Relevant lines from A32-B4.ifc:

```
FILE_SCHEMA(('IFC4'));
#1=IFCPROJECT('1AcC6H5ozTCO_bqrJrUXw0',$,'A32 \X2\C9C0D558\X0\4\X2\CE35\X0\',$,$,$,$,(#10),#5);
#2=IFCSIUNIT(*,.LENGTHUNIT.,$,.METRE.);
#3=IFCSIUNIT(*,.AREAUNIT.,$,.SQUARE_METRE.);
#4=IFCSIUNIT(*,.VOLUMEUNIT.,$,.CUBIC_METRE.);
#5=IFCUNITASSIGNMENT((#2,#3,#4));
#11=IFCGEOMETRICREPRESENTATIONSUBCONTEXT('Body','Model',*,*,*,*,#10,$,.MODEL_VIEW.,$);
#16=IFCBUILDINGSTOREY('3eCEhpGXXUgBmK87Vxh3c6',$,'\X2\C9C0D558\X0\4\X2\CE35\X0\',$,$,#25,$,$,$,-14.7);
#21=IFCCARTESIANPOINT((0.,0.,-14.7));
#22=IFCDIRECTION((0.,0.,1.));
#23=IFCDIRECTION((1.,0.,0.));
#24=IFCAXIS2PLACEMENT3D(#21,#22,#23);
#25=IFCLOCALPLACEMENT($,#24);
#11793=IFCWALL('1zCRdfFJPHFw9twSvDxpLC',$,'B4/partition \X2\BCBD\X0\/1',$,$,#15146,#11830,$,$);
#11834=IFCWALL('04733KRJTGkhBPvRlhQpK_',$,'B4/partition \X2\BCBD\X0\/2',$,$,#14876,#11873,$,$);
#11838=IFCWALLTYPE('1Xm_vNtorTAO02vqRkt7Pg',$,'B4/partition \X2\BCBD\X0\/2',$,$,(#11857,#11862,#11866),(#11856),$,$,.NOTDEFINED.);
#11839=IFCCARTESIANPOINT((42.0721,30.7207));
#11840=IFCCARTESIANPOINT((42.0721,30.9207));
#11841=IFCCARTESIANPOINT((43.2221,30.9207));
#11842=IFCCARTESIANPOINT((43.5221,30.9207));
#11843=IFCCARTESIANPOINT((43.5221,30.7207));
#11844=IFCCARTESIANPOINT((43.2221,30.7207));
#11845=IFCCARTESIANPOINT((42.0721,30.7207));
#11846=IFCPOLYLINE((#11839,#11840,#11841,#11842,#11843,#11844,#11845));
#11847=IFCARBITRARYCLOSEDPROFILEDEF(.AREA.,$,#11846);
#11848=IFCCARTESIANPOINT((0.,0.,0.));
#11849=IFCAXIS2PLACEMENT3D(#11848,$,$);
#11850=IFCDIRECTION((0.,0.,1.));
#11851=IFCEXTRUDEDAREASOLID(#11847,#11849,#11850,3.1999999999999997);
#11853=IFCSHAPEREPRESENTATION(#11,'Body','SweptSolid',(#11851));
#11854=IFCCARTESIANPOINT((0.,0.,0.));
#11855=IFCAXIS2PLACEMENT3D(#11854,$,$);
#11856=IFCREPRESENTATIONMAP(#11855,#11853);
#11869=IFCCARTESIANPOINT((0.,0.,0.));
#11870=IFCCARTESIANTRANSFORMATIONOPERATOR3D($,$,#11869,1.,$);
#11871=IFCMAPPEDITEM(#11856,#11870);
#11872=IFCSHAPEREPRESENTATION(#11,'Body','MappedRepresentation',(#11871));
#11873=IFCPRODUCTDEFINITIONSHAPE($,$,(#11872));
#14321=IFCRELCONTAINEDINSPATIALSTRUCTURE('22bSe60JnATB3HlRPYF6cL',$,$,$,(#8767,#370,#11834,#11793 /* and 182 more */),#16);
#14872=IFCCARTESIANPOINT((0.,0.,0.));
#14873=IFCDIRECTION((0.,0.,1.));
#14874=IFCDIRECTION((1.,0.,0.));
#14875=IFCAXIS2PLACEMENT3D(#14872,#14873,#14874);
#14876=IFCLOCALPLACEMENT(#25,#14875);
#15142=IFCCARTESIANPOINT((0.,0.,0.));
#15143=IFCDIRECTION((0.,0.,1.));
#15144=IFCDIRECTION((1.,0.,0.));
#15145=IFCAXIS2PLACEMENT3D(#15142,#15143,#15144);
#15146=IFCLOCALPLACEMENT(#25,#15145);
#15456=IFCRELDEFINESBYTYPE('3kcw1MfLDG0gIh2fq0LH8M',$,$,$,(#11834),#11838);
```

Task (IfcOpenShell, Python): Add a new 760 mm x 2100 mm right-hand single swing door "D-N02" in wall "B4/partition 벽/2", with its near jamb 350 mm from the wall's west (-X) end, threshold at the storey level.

```python
import numpy as np
import ifcopenshell
import ifcopenshell.api.feature
import ifcopenshell.api.geometry
import ifcopenshell.api.root
import ifcopenshell.api.spatial
import ifcopenshell.geom
import ifcopenshell.util.element
import ifcopenshell.util.placement
import ifcopenshell.util.representation
import ifcopenshell.util.shape
import ifcopenshell.util.unit

model = ifcopenshell.open("A32-B4.ifc")
unit_scale = ifcopenshell.util.unit.calculate_unit_scale(model)
settings = ifcopenshell.geom.settings()


def volume(element):
    """Net volume in cubic metres, openings subtracted."""
    shape = ifcopenshell.geom.create_shape(settings, element)
    return ifcopenshell.util.shape.get_volume(shape.geometry)


wall = model.by_id(11834)
storey = ifcopenshell.util.element.get_container(wall, ifc_class="IfcBuildingStorey")
context = ifcopenshell.util.representation.get_context(model, "Model", "Body", "MODEL_VIEW")
before = volume(wall)

width, height, from_end, sill = 0.76, 2.1, 0.35, 0.0  # metres

# The wall runs along its own X axis, and the end named is its -X end.
wall_shape = ifcopenshell.geom.create_shape(settings, wall)
x, y, z = ifcopenshell.util.shape.get_vertices(wall_shape.geometry).T
start = x.min() + from_end
face, thickness = float(y.min()), float(y.max() - y.min())
wall_matrix = ifcopenshell.util.placement.get_local_placement(wall.ObjectPlacement)
level = ifcopenshell.util.placement.get_local_placement(storey.ObjectPlacement)[2, 3]


def in_wall(x, y):
    """Placement at x, y metres in the wall's axes, at sill height."""
    matrix = wall_matrix.copy()
    matrix[:, 3] = wall_matrix @ np.array([x / unit_scale, y / unit_scale, 0.0, 1.0])
    matrix[2, 3] = level + sill / unit_scale
    return matrix


# Opening: a box that overshoots both wall faces by 50 mm.
opening = ifcopenshell.api.root.create_entity(model, ifc_class="IfcOpeningElement", predefined_type="OPENING")
box = ifcopenshell.api.geometry.add_wall_representation(
    model, context=context, length=width, height=height, thickness=thickness + 0.1
)
ifcopenshell.api.geometry.assign_representation(model, product=opening, representation=box)
ifcopenshell.api.geometry.edit_object_placement(model, product=opening, matrix=in_wall(start, face - 0.05), is_si=False)
ifcopenshell.api.feature.add_feature(model, feature=opening, element=wall)

door = ifcopenshell.api.root.create_entity(model, ifc_class="IfcDoor", name="D-N02", predefined_type="DOOR")
door.OverallWidth, door.OverallHeight = width / unit_scale, height / unit_scale
door.OperationType = "SINGLE_SWING_RIGHT"
body = ifcopenshell.api.geometry.add_door_representation(
    model,
    context=context,
    overall_width=door.OverallWidth,
    overall_height=door.OverallHeight,
    operation_type="SINGLE_SWING_RIGHT",
    lining_properties={"LiningDepth": thickness / unit_scale, "ThresholdDepth": thickness / unit_scale},
)
ifcopenshell.api.geometry.assign_representation(model, product=door, representation=body)
ifcopenshell.api.spatial.assign_container(model, products=[door], relating_structure=storey)
ifcopenshell.api.feature.add_filling(model, opening=opening, element=door)

# The lining spans the wall, so the door starts at the wall face.
ifcopenshell.api.geometry.edit_object_placement(model, product=door, matrix=in_wall(start, face), is_si=False)

after = volume(wall)

print(f"wall volume {before:.3f} -> {after:.3f} m3")

model.write("A32-B4_edited.ifc")
```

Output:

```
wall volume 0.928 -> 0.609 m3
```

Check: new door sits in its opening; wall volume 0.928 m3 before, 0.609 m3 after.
